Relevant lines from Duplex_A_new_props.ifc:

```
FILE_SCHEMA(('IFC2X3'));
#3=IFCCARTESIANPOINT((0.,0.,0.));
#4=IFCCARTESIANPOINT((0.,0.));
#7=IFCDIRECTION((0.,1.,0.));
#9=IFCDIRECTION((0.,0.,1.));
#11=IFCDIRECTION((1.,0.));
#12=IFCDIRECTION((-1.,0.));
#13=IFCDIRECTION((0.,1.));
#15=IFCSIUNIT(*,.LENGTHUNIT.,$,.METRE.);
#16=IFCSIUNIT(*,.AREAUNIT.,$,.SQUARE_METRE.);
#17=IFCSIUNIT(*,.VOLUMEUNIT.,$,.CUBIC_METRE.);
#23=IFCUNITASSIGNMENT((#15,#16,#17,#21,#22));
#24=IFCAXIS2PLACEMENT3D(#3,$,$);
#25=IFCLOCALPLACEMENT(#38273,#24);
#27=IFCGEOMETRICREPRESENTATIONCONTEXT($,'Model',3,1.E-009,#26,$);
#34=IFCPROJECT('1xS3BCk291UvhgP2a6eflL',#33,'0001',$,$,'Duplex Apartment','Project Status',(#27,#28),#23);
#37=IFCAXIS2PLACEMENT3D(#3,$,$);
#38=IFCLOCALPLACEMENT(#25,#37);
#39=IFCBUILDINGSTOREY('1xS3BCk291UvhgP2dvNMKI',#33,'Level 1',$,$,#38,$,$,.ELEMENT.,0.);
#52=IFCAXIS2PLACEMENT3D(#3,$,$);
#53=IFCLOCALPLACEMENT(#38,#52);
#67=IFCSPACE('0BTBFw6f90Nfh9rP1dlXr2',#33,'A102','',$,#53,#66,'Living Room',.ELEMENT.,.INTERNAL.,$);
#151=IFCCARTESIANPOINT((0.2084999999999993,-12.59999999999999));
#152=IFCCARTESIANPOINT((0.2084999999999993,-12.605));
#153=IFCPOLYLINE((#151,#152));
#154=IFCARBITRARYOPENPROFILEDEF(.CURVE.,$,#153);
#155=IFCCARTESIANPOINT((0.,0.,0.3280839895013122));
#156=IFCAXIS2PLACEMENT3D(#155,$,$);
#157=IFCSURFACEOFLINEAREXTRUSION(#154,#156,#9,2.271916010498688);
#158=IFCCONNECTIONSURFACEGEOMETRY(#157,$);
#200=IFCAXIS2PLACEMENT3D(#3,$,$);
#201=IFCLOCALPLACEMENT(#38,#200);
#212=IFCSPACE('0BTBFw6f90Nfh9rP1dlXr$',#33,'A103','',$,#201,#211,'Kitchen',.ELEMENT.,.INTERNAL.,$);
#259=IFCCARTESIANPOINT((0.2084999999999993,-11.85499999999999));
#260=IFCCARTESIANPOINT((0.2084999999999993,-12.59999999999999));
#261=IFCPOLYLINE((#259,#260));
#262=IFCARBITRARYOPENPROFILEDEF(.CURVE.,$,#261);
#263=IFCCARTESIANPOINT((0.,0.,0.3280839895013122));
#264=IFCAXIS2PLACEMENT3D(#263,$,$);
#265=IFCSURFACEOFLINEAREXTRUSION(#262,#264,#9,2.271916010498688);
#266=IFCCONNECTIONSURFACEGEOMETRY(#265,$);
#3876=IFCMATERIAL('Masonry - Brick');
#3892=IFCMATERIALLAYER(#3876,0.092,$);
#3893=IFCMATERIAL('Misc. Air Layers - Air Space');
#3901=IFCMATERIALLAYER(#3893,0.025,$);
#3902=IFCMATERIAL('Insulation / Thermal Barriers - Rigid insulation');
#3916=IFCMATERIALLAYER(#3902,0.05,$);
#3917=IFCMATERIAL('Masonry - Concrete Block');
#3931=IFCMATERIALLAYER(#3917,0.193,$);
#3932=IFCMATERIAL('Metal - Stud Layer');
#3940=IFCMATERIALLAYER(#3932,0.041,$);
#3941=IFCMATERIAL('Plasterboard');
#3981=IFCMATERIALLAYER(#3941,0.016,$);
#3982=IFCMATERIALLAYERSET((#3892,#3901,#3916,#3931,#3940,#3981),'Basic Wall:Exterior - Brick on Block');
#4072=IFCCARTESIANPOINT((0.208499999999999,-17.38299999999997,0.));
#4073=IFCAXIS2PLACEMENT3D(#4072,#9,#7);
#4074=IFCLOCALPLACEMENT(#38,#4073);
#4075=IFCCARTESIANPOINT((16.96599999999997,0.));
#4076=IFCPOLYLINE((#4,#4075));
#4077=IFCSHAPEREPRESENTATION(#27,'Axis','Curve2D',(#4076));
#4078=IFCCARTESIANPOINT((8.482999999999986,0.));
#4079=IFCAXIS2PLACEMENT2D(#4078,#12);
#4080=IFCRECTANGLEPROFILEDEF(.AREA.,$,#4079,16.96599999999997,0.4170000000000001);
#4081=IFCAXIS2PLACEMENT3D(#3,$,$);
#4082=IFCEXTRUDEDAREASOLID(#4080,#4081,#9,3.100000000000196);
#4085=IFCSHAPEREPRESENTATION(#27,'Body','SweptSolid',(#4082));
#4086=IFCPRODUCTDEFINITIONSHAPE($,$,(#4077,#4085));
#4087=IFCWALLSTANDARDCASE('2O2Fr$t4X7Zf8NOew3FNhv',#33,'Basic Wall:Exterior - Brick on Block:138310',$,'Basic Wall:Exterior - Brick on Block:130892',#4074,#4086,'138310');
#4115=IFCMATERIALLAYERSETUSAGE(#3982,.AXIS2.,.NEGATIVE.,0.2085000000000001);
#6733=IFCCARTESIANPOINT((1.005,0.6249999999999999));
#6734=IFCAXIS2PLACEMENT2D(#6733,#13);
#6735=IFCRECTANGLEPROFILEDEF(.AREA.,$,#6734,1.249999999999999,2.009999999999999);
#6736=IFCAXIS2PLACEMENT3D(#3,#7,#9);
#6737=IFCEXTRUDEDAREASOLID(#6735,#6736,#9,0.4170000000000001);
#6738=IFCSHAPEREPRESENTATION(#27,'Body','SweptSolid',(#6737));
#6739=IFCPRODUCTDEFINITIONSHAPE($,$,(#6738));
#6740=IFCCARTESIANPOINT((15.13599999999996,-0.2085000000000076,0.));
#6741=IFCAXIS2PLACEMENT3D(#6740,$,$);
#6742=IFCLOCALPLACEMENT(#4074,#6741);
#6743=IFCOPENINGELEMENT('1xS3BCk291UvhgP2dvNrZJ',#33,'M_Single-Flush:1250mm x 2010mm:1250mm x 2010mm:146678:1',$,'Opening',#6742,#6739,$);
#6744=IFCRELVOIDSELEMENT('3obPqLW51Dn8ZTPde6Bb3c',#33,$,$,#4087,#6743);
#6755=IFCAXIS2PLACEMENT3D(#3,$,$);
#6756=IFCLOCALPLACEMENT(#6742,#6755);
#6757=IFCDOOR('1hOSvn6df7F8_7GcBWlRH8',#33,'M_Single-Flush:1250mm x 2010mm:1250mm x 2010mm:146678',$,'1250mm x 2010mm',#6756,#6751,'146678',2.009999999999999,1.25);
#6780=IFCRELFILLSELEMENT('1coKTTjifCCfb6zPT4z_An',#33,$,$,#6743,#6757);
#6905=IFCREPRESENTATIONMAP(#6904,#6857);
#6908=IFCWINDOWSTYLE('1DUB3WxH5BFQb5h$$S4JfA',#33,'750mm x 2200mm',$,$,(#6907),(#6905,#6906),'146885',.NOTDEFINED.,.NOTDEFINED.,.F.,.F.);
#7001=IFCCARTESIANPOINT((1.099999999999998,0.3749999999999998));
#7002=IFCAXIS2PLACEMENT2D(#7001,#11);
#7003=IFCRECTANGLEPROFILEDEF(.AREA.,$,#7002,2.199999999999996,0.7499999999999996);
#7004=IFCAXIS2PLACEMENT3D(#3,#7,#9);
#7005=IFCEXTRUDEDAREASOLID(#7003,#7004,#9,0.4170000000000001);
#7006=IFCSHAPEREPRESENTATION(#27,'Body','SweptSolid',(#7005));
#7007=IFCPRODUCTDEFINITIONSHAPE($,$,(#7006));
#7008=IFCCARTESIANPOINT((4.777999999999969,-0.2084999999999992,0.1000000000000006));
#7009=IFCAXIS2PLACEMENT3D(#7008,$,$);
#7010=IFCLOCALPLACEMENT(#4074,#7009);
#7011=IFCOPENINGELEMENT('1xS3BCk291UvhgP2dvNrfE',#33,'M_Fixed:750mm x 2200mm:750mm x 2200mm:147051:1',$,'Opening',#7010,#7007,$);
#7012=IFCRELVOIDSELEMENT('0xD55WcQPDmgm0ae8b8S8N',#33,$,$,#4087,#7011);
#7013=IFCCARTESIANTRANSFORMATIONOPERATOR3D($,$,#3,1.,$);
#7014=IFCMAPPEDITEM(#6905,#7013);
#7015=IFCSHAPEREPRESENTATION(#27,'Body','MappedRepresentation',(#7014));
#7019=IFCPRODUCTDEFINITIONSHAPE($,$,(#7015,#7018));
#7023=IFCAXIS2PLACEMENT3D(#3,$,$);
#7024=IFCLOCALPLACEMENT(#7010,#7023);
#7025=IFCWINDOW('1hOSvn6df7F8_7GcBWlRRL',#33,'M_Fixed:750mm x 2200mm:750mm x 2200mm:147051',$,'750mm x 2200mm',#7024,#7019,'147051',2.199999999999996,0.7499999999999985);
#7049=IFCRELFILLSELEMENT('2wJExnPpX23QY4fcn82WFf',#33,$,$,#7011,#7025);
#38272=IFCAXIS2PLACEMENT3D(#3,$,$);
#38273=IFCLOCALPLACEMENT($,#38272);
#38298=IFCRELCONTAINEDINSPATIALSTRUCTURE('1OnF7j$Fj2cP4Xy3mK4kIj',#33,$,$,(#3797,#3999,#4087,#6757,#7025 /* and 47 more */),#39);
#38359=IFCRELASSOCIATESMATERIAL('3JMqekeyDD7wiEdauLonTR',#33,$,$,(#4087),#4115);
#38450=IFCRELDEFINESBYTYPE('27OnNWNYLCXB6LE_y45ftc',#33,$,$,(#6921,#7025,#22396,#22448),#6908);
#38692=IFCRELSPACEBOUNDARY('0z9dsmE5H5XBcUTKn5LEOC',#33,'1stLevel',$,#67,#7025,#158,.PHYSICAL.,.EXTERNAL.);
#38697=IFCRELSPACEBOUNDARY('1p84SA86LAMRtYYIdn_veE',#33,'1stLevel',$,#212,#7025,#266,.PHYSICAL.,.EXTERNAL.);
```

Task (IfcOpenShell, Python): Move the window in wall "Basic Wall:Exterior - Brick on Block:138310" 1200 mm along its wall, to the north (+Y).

```python
import numpy as np
import ifcopenshell
import ifcopenshell.api.geometry
import ifcopenshell.util.placement

model = ifcopenshell.open("Duplex_A_new_props.ifc")

window = model.by_id(7025)
opening = window.FillsVoids[0].RelatingOpeningElement
wall = opening.VoidsElements[0].RelatingBuildingElement

wall_matrix = ifcopenshell.util.placement.get_local_placement(wall.ObjectPlacement)
shift = wall_matrix[:3, 0] * 1.2
before = ifcopenshell.util.placement.get_local_placement(window.ObjectPlacement)[:3, 3].copy()

# The window is placed relative to its opening, so it follows when the opening moves.
matrix = ifcopenshell.util.placement.get_local_placement(opening.ObjectPlacement)
matrix[:3, 3] += shift
ifcopenshell.api.geometry.edit_object_placement(
    model, product=opening, matrix=matrix, is_si=False, should_transform_children=True
)

# Space boundary surfaces are stored in each space's coordinates; move them too.
for rel in window.ProvidesBoundaries:
    if not rel.ConnectionGeometry:
        continue
    surface = rel.ConnectionGeometry.SurfaceOnRelatingElement
    space_matrix = ifcopenshell.util.placement.get_local_placement(rel.RelatingSpace.ObjectPlacement)
    point = np.array(surface.Position.Location.Coordinates) + space_matrix[:3, :3].T @ shift
    surface.Position = model.createIfcAxis2Placement3D(
        model.createIfcCartesianPoint(point.tolist()), surface.Position.Axis, surface.Position.RefDirection
    )

after = ifcopenshell.util.placement.get_local_placement(window.ObjectPlacement)[:3, 3]
print("window moved by", (after - before).round(3) + 0.0)

model.write("Duplex_A_new_props-out.ifc")
```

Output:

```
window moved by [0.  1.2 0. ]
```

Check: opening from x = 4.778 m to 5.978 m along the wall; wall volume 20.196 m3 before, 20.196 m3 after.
